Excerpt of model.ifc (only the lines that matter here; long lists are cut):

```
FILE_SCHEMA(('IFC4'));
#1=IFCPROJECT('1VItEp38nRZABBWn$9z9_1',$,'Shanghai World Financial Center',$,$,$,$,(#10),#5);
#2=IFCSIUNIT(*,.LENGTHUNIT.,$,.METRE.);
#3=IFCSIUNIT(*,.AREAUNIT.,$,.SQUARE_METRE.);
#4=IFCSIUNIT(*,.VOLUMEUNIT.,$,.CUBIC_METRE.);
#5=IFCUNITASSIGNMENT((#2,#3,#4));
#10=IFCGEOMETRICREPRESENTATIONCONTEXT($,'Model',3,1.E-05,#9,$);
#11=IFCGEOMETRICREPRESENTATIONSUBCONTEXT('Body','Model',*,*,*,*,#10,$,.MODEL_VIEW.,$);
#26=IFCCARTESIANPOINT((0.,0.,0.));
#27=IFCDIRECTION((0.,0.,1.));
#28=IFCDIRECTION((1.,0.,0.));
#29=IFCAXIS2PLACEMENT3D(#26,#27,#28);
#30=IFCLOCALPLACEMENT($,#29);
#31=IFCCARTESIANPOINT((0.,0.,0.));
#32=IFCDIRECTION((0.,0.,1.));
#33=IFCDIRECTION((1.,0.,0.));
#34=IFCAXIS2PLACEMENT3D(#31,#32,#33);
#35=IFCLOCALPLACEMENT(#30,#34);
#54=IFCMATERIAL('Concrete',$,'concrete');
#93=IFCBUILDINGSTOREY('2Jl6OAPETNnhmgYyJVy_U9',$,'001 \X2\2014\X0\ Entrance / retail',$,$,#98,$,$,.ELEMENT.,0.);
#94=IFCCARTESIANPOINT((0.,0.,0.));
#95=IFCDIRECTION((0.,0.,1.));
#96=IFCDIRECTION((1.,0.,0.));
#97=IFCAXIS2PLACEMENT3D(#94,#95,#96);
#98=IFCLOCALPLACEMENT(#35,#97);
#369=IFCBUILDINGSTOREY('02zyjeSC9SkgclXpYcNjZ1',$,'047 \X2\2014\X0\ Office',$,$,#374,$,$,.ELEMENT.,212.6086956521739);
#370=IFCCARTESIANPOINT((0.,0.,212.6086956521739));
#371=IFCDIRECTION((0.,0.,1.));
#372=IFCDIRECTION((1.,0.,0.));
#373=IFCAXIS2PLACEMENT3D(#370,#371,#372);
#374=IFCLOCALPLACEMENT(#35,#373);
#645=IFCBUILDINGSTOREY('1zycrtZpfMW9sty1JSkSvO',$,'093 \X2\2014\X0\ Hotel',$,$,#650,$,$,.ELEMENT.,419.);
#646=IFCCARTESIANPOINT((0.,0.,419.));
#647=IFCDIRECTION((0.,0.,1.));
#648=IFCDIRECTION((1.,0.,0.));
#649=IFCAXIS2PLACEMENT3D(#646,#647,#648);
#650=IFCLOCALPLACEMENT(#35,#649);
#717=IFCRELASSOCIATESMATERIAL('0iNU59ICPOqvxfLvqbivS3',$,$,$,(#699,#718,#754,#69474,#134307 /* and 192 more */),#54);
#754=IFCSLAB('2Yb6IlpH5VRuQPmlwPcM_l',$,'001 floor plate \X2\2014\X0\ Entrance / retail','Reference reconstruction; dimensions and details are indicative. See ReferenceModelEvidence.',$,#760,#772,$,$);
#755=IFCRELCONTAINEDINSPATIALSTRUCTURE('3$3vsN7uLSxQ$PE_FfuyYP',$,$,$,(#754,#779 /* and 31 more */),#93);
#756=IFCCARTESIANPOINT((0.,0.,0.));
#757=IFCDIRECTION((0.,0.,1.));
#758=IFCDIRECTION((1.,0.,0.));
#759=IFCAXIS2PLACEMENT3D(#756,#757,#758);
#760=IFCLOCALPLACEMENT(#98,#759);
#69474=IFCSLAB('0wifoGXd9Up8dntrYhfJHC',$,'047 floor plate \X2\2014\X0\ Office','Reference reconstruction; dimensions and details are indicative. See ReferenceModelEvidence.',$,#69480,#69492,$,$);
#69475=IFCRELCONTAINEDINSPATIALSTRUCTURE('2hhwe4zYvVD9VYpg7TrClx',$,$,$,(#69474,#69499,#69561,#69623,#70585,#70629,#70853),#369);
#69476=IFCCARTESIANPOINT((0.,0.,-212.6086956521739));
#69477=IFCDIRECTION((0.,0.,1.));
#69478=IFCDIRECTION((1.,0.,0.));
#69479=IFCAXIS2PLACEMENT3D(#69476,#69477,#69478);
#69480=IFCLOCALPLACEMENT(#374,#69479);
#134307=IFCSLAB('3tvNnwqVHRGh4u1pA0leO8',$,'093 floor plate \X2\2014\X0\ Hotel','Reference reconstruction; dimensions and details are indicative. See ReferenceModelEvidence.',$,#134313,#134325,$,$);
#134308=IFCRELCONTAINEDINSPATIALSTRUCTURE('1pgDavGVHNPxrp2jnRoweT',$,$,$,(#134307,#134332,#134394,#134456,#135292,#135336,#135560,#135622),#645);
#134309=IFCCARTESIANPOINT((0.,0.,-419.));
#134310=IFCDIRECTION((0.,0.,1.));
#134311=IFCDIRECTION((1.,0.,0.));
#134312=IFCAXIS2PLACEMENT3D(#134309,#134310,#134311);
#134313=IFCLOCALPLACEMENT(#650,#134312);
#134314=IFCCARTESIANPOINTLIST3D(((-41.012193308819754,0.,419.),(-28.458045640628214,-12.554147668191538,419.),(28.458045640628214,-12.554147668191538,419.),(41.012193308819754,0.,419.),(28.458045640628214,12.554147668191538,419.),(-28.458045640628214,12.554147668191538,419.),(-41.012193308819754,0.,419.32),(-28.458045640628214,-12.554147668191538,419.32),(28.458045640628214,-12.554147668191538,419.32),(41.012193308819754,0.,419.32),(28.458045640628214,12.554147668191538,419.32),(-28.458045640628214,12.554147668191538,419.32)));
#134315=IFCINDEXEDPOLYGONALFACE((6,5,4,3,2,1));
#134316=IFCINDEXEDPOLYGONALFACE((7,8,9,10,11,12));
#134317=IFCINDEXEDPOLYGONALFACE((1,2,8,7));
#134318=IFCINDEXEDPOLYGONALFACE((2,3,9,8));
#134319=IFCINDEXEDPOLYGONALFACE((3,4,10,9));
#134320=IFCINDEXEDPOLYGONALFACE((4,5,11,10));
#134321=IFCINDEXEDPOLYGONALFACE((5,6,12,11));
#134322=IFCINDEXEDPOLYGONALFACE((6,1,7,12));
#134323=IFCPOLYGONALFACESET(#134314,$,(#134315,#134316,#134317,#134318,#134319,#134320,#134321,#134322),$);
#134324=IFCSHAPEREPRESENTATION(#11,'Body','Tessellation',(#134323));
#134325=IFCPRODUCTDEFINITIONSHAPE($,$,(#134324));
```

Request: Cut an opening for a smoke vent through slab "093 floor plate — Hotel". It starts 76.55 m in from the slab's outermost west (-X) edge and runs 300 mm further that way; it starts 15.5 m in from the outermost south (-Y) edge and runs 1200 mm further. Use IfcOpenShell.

```python
import numpy as np
import ifcopenshell
import ifcopenshell.api.feature
import ifcopenshell.api.geometry
import ifcopenshell.api.root
import ifcopenshell.geom
import ifcopenshell.util.placement
import ifcopenshell.util.representation
import ifcopenshell.util.shape
import ifcopenshell.util.unit

model = ifcopenshell.open("model.ifc")
unit_scale = ifcopenshell.util.unit.calculate_unit_scale(model)
settings = ifcopenshell.geom.settings()


def volume(element):
    """Net volume in cubic metres, openings subtracted."""
    shape = ifcopenshell.geom.create_shape(settings, element)
    return ifcopenshell.util.shape.get_volume(shape.geometry)


slab = model.by_id(134307)
before = volume(slab)

# Extent in the slab's own axes, in metres. The edges named are its -X and -Y sides.
slab_shape = ifcopenshell.geom.create_shape(settings, slab)
vertices = ifcopenshell.util.shape.get_vertices(slab_shape.geometry)
x_min, y_min, bottom = vertices.min(axis=0)
top = vertices[:, 2].max()

opening = ifcopenshell.api.root.create_entity(model, ifc_class="IfcOpeningElement", name="Smoke vent opening", predefined_type="OPENING")
context = ifcopenshell.util.representation.get_context(model, "Model", "Body", "MODEL_VIEW")
width, depth = 0.3, 1.2
outline = [(0.0, 0.0), (width, 0.0), (width, depth), (0.0, depth), (0.0, 0.0)]
# Overshoot both faces by 50 mm so the cut is clean.
shape = ifcopenshell.api.geometry.add_slab_representation(
    model, context=context, depth=top - bottom + 0.1, polyline=outline
)
ifcopenshell.api.geometry.assign_representation(model, product=opening, representation=shape)

matrix = ifcopenshell.util.placement.get_local_placement(slab.ObjectPlacement)
matrix[:, 3] = matrix @ np.append(np.array([x_min + 76.55, y_min + 15.5, bottom - 0.05]) / unit_scale, 1.0)
ifcopenshell.api.geometry.edit_object_placement(model, product=opening, matrix=matrix, is_si=False)
ifcopenshell.api.feature.add_feature(model, feature=opening, element=slab)

after = volume(slab)

print(f"slab volume {before:.3f} -> {after:.3f} m3")

model.write("model_rev.ifc")
```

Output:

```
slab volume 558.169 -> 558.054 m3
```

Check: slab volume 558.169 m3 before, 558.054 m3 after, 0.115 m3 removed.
